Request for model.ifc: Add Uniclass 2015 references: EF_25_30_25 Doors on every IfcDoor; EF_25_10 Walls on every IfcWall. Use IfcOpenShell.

First a look at what the model holds.

```python
import ifcopenshell

model = ifcopenshell.open("model.ifc")
print(model.schema)
print("classifications:", [c.Name for c in model.by_type("IfcClassification")])
for ifc_class in ("IfcDoor", "IfcRoof", "IfcStair", "IfcWall", "IfcWindow"):
    print(ifc_class, len(model.by_type(ifc_class)))
```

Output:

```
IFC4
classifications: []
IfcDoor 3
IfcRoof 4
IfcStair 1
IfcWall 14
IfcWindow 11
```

```python
import ifcopenshell
import ifcopenshell.api.classification

model = ifcopenshell.open("model.ifc")

system = ifcopenshell.api.classification.add_classification(model, classification="Uniclass 2015")

codes = {
    "IfcDoor": ("EF_25_30_25", "Doors"),
    "IfcWall": ("EF_25_10", "Walls"),
}
for ifc_class, (code, name) in codes.items():
    products = model.by_type(ifc_class)
    ifcopenshell.api.classification.add_reference(
        model, products=products, classification=system, identification=code, name=name
    )
    print(code, len(products))

model.write("model_rev.ifc")
```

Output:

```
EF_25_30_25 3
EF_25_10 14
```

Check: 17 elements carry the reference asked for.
